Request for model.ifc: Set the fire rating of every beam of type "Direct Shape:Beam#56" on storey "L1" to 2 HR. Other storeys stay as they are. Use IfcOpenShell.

First a look at what the model holds.

```python
import ifcopenshell
import ifcopenshell.util.element

model = ifcopenshell.open("model.ifc")
print(model.schema)
storey = next(s for s in model.by_type("IfcBuildingStorey") if s.Name == "L1")
beams = [e for e in ifcopenshell.util.element.get_decomposition(storey) if e.is_a("IfcBeam")]
seen = {}
for e in beams:
    element_type = ifcopenshell.util.element.get_type(e)
    key = (element_type.Name if element_type != e and element_type else None, ifcopenshell.util.element.get_pset(e, "Pset_BeamCommon", "FireRating"))
    seen[key] = seen.get(key, 0) + 1
for (name, value), count in sorted(seen.items(), key=str):
    print(count, "x", name, "|", value)
```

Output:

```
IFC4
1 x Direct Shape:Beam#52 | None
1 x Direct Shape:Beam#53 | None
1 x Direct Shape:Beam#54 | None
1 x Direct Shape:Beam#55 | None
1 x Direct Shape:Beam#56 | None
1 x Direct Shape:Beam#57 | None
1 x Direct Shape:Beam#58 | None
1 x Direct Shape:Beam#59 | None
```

```python
import ifcopenshell
import ifcopenshell.api.pset
import ifcopenshell.util.element

model = ifcopenshell.open("model.ifc")

storey = next(s for s in model.by_type("IfcBuildingStorey") if s.Name == "L1")
beams = [e for e in ifcopenshell.util.element.get_decomposition(storey) if e.is_a("IfcBeam")]

count = 0
for e in beams:
    element_type = ifcopenshell.util.element.get_type(e)
    if element_type in (None, e) or element_type.Name != "Direct Shape:Beam#56":
        continue
    # add_pset returns the element's existing set when there is one.
    pset = ifcopenshell.api.pset.add_pset(model, product=e, name="Pset_BeamCommon")
    ifcopenshell.api.pset.edit_pset(model, pset=pset, properties={"FireRating": "2 HR"})
    count += 1

print(count, "beams updated")

model.write("model_rev.ifc")
```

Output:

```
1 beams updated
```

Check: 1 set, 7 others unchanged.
